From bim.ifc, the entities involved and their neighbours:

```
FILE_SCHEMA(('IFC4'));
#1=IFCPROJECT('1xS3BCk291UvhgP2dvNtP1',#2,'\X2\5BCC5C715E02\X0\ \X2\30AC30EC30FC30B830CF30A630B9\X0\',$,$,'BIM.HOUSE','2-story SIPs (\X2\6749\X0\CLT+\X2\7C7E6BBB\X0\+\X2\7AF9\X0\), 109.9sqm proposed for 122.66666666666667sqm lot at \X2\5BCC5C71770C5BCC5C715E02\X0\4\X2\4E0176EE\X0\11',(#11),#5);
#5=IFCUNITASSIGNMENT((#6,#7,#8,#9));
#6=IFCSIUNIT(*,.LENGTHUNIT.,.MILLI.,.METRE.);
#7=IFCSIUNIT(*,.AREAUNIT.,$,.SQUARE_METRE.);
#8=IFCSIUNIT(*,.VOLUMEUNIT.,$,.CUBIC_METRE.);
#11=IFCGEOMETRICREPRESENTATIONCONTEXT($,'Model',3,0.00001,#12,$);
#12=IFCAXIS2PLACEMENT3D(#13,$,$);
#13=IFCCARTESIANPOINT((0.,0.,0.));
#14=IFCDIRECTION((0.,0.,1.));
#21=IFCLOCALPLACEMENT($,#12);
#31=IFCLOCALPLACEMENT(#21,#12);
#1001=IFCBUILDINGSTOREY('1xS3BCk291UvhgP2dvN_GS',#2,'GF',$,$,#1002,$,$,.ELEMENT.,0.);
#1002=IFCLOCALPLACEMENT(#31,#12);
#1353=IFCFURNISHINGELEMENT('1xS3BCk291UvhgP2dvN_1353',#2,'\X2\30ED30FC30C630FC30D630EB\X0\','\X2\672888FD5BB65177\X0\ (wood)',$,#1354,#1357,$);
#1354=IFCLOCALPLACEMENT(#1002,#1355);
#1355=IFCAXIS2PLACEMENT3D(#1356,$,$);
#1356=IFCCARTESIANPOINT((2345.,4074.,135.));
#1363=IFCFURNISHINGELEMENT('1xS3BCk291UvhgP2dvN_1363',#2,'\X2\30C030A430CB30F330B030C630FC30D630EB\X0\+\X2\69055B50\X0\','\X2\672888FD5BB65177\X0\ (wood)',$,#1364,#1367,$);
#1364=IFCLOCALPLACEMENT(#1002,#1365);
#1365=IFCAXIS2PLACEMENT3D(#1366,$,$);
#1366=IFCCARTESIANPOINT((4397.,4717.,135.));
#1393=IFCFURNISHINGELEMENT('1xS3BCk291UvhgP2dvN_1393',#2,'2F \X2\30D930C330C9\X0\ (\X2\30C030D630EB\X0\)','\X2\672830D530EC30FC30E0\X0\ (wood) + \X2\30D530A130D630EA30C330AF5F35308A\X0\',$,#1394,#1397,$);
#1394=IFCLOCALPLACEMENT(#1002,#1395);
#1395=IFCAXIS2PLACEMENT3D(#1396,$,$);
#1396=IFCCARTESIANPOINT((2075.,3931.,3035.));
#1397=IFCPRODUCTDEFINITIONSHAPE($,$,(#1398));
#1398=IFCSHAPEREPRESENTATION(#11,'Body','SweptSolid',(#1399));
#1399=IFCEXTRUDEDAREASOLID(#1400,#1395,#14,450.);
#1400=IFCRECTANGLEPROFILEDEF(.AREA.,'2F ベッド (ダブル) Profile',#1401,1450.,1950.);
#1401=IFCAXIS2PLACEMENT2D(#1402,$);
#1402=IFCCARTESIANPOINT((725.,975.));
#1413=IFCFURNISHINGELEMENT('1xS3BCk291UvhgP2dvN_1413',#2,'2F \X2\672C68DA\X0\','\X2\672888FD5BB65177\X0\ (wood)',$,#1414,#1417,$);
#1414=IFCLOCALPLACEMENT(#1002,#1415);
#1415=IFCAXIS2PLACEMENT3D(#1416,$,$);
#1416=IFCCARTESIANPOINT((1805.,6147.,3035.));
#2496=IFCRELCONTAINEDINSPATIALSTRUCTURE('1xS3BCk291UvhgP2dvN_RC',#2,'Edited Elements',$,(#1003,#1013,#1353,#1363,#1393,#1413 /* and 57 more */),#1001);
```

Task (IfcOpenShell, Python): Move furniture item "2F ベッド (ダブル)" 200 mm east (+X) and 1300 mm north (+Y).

```python
import ifcopenshell
import ifcopenshell.api.geometry
import ifcopenshell.util.placement
import ifcopenshell.util.unit

model = ifcopenshell.open("bim.ifc")
unit_scale = ifcopenshell.util.unit.calculate_unit_scale(model)

item = model.by_guid("1xS3BCk291UvhgP2dvN_1393")
matrix = ifcopenshell.util.placement.get_local_placement(item.ObjectPlacement)
matrix[0, 3] += 0.2 / unit_scale
matrix[1, 3] += 1.3 / unit_scale
ifcopenshell.api.geometry.edit_object_placement(model, product=item, matrix=matrix, is_si=False)

print(ifcopenshell.util.placement.get_local_placement(item.ObjectPlacement).round(3) + 0.0)

model.write("bim_rev.ifc")
```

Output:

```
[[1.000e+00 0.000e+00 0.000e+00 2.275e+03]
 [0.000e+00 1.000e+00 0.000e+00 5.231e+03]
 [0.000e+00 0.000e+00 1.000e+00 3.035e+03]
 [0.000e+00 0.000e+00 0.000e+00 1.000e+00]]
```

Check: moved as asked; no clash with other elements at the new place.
